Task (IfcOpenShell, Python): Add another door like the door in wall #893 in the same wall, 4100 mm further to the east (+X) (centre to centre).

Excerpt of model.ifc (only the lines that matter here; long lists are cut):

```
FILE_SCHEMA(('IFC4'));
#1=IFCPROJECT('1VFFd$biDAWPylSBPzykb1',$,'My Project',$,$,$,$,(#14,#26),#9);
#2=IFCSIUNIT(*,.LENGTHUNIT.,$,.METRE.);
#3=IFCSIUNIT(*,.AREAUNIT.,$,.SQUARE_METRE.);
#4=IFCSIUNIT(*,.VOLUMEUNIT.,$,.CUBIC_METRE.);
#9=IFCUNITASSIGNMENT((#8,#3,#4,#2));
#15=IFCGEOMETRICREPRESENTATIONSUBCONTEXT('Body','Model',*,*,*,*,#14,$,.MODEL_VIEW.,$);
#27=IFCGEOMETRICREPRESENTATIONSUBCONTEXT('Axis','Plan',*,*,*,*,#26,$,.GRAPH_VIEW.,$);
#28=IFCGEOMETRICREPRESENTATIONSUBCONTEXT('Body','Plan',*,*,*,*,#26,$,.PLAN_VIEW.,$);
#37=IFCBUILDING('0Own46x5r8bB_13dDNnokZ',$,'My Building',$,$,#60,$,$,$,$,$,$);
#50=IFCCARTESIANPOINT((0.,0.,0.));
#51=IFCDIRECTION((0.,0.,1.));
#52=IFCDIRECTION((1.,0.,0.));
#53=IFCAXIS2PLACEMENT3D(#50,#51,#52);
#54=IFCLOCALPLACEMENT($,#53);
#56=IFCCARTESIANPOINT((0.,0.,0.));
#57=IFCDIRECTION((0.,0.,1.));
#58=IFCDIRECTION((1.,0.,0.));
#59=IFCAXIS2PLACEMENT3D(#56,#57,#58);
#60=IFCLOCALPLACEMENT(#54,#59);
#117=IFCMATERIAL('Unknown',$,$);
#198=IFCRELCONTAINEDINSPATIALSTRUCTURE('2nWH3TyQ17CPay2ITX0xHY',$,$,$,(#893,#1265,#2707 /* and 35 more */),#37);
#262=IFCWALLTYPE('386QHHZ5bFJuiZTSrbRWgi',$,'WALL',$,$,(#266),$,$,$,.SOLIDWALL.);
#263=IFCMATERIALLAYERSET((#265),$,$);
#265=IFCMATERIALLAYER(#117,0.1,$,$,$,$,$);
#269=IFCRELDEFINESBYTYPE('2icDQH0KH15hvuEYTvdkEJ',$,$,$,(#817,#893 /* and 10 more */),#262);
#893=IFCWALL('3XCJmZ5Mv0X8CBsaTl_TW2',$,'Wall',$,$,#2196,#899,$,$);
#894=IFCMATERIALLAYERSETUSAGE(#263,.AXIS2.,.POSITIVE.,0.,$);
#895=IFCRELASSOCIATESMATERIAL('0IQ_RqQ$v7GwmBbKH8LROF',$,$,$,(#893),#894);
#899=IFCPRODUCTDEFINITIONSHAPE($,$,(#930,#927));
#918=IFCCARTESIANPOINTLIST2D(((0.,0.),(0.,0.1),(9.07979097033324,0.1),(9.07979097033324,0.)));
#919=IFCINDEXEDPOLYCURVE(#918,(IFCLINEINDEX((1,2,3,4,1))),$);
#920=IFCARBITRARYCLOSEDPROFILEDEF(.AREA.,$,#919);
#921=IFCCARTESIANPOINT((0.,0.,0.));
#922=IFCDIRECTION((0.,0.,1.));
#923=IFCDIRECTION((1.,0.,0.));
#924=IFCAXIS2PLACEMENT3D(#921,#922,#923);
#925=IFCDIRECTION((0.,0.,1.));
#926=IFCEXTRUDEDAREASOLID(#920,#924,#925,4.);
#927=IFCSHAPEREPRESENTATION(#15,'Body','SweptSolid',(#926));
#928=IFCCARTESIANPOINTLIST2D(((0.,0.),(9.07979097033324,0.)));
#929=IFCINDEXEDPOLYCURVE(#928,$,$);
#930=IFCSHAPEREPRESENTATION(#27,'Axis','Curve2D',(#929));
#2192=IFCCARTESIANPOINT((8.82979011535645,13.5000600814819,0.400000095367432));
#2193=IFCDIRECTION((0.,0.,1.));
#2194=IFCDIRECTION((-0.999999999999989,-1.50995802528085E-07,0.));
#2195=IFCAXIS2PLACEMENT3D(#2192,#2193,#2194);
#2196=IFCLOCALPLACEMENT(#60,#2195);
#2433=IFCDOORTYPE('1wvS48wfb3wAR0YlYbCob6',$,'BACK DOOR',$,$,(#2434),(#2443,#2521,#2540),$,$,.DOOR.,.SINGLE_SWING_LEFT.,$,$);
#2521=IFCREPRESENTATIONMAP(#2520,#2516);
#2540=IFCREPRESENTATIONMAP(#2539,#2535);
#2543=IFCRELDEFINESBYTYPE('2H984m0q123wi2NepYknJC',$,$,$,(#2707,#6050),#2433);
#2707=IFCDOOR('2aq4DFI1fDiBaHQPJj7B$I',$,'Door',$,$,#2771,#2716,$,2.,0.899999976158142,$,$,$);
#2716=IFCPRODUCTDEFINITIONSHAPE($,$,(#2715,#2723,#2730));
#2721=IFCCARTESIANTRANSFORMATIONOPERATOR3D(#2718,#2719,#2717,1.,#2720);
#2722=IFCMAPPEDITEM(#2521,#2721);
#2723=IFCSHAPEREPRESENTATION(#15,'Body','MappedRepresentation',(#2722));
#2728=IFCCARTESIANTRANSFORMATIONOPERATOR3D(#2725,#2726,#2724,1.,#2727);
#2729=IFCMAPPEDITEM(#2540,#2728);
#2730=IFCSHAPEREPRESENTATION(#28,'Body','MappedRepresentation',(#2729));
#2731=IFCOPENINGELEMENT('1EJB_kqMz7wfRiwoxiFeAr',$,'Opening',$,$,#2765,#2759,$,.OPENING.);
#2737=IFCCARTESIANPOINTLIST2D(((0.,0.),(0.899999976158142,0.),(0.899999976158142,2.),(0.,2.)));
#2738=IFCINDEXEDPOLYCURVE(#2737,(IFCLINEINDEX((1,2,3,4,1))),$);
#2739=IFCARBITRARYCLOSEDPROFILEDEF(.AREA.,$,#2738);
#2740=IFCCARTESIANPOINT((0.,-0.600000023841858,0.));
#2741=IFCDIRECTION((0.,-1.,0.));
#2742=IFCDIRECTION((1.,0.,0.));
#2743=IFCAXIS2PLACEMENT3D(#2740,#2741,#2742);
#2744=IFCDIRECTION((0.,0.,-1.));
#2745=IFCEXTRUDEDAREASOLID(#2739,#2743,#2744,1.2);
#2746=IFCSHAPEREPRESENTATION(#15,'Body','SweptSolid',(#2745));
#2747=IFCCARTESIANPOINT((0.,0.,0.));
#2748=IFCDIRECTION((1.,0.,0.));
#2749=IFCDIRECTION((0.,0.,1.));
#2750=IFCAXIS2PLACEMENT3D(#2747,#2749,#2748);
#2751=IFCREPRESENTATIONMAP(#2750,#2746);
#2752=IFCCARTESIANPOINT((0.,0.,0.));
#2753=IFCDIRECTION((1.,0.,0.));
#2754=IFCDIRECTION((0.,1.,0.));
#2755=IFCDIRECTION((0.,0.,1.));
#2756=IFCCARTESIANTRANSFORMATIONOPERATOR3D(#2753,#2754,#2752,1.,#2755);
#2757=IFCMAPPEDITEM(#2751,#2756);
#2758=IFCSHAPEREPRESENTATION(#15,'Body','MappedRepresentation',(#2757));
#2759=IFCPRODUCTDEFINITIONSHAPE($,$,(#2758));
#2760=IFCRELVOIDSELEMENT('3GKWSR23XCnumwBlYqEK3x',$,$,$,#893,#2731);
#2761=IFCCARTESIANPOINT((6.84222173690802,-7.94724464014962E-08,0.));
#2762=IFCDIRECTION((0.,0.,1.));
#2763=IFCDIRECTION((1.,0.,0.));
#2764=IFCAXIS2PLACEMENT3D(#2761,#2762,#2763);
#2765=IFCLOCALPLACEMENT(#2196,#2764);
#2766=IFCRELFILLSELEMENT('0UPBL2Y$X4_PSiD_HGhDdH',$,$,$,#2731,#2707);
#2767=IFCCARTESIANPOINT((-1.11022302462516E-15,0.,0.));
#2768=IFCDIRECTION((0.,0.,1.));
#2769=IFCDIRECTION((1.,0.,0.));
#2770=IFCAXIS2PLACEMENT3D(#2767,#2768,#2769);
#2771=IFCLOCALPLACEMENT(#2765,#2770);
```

```python
import ifcopenshell
import ifcopenshell.api.feature
import ifcopenshell.api.geometry
import ifcopenshell.api.root
import ifcopenshell.geom
import ifcopenshell.util.element
import ifcopenshell.util.placement
import ifcopenshell.util.shape
import ifcopenshell.util.unit

model = ifcopenshell.open("model.ifc")
unit_scale = ifcopenshell.util.unit.calculate_unit_scale(model)
settings = ifcopenshell.geom.settings()


def volume(element):
    """Net volume in cubic metres, openings subtracted."""
    shape = ifcopenshell.geom.create_shape(settings, element)
    return ifcopenshell.util.shape.get_volume(shape.geometry)


door = model.by_guid("2aq4DFI1fDiBaHQPJj7B$I")
opening = door.FillsVoids[0].RelatingOpeningElement
wall = opening.VoidsElements[0].RelatingBuildingElement
before = volume(wall)
shift = ifcopenshell.util.placement.get_local_placement(wall.ObjectPlacement)[:3, 0] * -4.1 / unit_scale

# copy_class copies the void relationship, type, container and properties, but no geometry.
new_opening = ifcopenshell.api.root.copy_class(model, product=opening)
new_opening.Representation = ifcopenshell.util.element.copy_deep(
    model, opening.Representation, exclude=["IfcGeometricRepresentationContext", "IfcRepresentationMap"]
)
new_door = ifcopenshell.api.root.copy_class(model, product=door)
new_door.Representation = ifcopenshell.util.element.copy_deep(
    model, door.Representation, exclude=["IfcGeometricRepresentationContext", "IfcRepresentationMap"]
)
ifcopenshell.api.feature.add_filling(model, opening=new_opening, element=new_door)

for old, new in ((opening, new_opening), (door, new_door)):
    matrix = ifcopenshell.util.placement.get_local_placement(old.ObjectPlacement)
    matrix[:3, 3] += shift
    ifcopenshell.api.geometry.edit_object_placement(model, product=new, matrix=matrix, is_si=False)

after = volume(wall)

print(f"wall volume {before:.3f} -> {after:.3f} m3")

model.write("model_updated.ifc")
```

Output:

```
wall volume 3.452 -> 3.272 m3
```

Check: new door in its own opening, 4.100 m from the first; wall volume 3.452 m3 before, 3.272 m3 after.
